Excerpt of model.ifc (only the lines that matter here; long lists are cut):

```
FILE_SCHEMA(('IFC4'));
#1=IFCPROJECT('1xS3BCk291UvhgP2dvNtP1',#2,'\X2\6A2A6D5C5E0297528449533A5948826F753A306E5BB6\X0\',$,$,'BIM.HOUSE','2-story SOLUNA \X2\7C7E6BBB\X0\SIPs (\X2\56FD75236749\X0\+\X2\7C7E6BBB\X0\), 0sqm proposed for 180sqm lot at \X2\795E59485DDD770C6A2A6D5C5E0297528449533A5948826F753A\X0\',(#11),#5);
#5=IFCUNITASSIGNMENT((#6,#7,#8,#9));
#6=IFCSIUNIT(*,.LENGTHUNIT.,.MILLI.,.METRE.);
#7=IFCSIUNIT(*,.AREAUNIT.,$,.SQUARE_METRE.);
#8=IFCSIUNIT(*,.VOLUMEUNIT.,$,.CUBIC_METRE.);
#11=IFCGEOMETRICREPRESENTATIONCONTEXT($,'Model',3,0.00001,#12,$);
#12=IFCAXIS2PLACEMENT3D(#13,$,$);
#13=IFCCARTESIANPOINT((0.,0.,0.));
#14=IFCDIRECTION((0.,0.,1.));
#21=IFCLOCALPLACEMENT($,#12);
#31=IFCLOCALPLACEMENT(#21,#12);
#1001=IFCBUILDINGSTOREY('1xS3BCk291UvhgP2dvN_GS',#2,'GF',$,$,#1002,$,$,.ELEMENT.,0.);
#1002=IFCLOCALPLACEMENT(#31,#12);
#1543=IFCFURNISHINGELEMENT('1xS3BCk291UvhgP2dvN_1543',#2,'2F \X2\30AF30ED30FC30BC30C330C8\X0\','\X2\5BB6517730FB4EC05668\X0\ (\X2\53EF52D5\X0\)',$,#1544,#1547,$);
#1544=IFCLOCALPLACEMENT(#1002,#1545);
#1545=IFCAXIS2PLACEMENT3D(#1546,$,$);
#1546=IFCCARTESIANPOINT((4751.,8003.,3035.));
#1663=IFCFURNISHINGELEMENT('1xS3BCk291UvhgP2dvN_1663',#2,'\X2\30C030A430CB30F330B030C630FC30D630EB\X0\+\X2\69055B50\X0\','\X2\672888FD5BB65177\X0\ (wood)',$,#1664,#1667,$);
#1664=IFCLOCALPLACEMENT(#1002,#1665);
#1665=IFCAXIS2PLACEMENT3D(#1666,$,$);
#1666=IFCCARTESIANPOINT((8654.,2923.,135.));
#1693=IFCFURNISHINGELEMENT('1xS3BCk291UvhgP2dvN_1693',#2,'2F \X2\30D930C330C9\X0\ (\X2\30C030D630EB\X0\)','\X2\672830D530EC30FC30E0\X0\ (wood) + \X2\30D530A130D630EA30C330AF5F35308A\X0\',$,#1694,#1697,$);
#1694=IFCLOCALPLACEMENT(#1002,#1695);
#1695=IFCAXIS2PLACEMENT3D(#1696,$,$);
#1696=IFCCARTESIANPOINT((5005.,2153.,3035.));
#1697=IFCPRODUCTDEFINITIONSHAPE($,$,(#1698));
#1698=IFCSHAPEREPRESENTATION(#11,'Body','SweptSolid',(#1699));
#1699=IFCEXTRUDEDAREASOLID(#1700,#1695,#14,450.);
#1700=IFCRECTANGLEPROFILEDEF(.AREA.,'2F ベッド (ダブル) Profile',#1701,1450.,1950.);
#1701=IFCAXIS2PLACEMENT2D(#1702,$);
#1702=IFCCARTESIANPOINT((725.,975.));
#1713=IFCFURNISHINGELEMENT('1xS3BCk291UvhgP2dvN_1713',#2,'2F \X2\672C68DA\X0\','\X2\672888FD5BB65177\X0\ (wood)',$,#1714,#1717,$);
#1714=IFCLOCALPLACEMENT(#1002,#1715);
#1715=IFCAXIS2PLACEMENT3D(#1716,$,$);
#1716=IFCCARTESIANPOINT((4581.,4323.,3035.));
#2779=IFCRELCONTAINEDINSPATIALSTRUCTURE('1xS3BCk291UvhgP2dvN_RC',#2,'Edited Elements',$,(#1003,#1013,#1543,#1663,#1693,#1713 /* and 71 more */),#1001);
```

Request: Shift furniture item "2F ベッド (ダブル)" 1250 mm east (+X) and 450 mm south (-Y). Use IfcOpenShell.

```python
import ifcopenshell
import ifcopenshell.api.geometry
import ifcopenshell.util.placement

model = ifcopenshell.open("model.ifc")

item = model.by_id(1693)
matrix = ifcopenshell.util.placement.get_local_placement(item.ObjectPlacement)
matrix[0, 3] += 1250.0
matrix[1, 3] -= 450.0
ifcopenshell.api.geometry.edit_object_placement(model, product=item, matrix=matrix, is_si=False)

print(ifcopenshell.util.placement.get_local_placement(item.ObjectPlacement).round(3) + 0.0)

model.write("model_updated.ifc")
```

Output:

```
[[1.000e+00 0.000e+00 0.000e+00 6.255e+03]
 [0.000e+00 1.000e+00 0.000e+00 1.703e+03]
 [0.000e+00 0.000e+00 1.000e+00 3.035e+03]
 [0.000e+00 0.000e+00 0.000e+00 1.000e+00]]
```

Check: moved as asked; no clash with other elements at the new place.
